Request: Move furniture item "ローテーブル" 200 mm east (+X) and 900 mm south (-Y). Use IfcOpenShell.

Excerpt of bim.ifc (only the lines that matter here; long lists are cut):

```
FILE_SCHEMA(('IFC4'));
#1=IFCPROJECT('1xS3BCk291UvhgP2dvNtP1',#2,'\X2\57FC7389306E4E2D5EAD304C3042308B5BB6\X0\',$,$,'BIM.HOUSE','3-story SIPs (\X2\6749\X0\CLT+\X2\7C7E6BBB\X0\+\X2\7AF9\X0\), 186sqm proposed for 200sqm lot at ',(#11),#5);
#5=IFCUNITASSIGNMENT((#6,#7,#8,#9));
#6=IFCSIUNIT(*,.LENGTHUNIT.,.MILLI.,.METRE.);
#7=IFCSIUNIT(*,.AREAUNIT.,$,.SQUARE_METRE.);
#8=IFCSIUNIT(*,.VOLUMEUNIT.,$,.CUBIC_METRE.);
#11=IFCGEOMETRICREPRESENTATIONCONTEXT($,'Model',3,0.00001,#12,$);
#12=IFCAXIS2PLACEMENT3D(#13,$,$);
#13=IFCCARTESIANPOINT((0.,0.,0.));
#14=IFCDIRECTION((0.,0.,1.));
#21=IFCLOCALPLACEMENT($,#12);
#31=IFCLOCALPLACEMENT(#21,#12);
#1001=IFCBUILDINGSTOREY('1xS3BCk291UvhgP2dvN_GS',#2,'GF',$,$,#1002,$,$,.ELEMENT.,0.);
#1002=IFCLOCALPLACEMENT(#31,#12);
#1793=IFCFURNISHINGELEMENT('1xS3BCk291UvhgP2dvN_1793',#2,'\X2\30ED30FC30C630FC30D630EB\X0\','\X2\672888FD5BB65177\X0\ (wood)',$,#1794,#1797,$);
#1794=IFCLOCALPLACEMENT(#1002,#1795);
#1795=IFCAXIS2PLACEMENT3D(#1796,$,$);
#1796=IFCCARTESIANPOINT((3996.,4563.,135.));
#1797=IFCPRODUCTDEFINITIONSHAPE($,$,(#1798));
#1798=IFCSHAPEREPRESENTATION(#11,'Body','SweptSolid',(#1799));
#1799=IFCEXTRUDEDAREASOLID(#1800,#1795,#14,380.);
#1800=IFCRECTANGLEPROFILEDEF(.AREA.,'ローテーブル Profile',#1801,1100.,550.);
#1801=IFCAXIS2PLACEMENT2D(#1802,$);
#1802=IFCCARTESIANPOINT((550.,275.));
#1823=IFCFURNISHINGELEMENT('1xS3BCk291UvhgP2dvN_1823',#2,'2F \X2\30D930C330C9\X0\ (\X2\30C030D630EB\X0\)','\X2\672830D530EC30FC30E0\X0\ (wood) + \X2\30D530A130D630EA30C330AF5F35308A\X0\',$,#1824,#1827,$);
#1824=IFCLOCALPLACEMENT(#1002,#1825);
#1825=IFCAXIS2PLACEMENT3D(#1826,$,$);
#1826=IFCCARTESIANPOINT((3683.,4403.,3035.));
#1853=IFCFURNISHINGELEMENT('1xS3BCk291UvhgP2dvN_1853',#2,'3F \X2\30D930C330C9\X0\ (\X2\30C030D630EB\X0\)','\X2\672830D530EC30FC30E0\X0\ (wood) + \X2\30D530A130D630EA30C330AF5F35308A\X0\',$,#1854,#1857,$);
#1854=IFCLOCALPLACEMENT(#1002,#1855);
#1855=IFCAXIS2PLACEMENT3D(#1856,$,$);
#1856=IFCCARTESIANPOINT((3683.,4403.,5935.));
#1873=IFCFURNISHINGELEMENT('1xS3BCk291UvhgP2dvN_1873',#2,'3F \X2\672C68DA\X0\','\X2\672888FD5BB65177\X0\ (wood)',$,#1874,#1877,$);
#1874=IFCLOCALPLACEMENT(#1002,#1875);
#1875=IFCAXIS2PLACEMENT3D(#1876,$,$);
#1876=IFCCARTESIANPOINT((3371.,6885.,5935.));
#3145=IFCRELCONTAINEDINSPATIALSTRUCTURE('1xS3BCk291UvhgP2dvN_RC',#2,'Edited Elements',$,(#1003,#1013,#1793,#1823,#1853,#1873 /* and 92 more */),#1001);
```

```python
import ifcopenshell
import ifcopenshell.api.geometry
import ifcopenshell.util.placement
import ifcopenshell.util.unit

model = ifcopenshell.open("bim.ifc")
unit_scale = ifcopenshell.util.unit.calculate_unit_scale(model)

item = model.by_guid("1xS3BCk291UvhgP2dvN_1793")
matrix = ifcopenshell.util.placement.get_local_placement(item.ObjectPlacement)
matrix[0, 3] += 0.2 / unit_scale
matrix[1, 3] -= 0.9 / unit_scale
ifcopenshell.api.geometry.edit_object_placement(model, product=item, matrix=matrix, is_si=False)

print(ifcopenshell.util.placement.get_local_placement(item.ObjectPlacement).round(3) + 0.0)

model.write("bim-out.ifc")
```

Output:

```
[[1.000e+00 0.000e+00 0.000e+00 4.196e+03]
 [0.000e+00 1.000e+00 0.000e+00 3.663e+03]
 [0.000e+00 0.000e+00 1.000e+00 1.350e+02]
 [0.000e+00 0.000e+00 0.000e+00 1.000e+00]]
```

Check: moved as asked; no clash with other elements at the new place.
